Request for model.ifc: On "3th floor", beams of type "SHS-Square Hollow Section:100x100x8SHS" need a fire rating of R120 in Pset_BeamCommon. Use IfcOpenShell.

First a look at what the model holds.

```python
import ifcopenshell
import ifcopenshell.util.element

model = ifcopenshell.open("model.ifc")
print(model.schema)
storey = next(s for s in model.by_type("IfcBuildingStorey") if s.Name == "3th floor")
beams = [e for e in ifcopenshell.util.element.get_decomposition(storey) if e.is_a("IfcBeam")]
seen = {}
for e in beams:
    element_type = ifcopenshell.util.element.get_type(e)
    key = (element_type.Name if element_type != e and element_type else None, ifcopenshell.util.element.get_pset(e, "Pset_BeamCommon", "FireRating"))
    seen[key] = seen.get(key, 0) + 1
for (name, value), count in sorted(seen.items(), key=str):
    print(count, "x", name, "|", value)
```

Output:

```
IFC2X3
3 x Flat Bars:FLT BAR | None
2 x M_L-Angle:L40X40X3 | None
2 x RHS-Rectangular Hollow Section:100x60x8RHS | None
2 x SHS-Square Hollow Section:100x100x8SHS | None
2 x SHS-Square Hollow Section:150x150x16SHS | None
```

```python
import ifcopenshell
import ifcopenshell.api.pset
import ifcopenshell.util.element

model = ifcopenshell.open("model.ifc")

storey = next(s for s in model.by_type("IfcBuildingStorey") if s.Name == "3th floor")
beams = [e for e in ifcopenshell.util.element.get_decomposition(storey) if e.is_a("IfcBeam")]

count = 0
for e in beams:
    element_type = ifcopenshell.util.element.get_type(e)
    if element_type in (None, e) or element_type.Name != "SHS-Square Hollow Section:100x100x8SHS":
        continue
    # add_pset returns the element's existing set when there is one.
    pset = ifcopenshell.api.pset.add_pset(model, product=e, name="Pset_BeamCommon")
    ifcopenshell.api.pset.edit_pset(model, pset=pset, properties={"FireRating": "R120"})
    count += 1

print(count, "beams updated")

model.write("model_updated.ifc")
```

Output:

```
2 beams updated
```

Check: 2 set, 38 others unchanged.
